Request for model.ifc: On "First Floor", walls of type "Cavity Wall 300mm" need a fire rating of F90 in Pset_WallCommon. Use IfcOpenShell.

First a look at what the model holds.

```python
import ifcopenshell
import ifcopenshell.util.element

model = ifcopenshell.open("model.ifc")
print(model.schema)
storey = next(s for s in model.by_type("IfcBuildingStorey") if s.Name == "First Floor")
walls = [e for e in ifcopenshell.util.element.get_decomposition(storey) if e.is_a("IfcWall")]
seen = {}
for e in walls:
    element_type = ifcopenshell.util.element.get_type(e)
    key = (element_type.Name if element_type != e and element_type else None, ifcopenshell.util.element.get_pset(e, "Pset_WallCommon", "FireRating"))
    seen[key] = seen.get(key, 0) + 1
for (name, value), count in sorted(seen.items(), key=str):
    print(count, "x", name, "|", value)
```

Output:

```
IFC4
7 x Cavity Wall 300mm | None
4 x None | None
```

```python
import ifcopenshell
import ifcopenshell.api.pset
import ifcopenshell.util.element

model = ifcopenshell.open("model.ifc")

storey = next(s for s in model.by_type("IfcBuildingStorey") if s.Name == "First Floor")
walls = [e for e in ifcopenshell.util.element.get_decomposition(storey) if e.is_a("IfcWall")]

count = 0
for e in walls:
    element_type = ifcopenshell.util.element.get_type(e)
    if element_type in (None, e) or element_type.Name != "Cavity Wall 300mm":
        continue
    # add_pset returns the element's existing set when there is one.
    pset = ifcopenshell.api.pset.add_pset(model, product=e, name="Pset_WallCommon")
    ifcopenshell.api.pset.edit_pset(model, pset=pset, properties={"FireRating": "F90"})
    count += 1

print(count, "walls updated")

model.write("model_updated.ifc")
```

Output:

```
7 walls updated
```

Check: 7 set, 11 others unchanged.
